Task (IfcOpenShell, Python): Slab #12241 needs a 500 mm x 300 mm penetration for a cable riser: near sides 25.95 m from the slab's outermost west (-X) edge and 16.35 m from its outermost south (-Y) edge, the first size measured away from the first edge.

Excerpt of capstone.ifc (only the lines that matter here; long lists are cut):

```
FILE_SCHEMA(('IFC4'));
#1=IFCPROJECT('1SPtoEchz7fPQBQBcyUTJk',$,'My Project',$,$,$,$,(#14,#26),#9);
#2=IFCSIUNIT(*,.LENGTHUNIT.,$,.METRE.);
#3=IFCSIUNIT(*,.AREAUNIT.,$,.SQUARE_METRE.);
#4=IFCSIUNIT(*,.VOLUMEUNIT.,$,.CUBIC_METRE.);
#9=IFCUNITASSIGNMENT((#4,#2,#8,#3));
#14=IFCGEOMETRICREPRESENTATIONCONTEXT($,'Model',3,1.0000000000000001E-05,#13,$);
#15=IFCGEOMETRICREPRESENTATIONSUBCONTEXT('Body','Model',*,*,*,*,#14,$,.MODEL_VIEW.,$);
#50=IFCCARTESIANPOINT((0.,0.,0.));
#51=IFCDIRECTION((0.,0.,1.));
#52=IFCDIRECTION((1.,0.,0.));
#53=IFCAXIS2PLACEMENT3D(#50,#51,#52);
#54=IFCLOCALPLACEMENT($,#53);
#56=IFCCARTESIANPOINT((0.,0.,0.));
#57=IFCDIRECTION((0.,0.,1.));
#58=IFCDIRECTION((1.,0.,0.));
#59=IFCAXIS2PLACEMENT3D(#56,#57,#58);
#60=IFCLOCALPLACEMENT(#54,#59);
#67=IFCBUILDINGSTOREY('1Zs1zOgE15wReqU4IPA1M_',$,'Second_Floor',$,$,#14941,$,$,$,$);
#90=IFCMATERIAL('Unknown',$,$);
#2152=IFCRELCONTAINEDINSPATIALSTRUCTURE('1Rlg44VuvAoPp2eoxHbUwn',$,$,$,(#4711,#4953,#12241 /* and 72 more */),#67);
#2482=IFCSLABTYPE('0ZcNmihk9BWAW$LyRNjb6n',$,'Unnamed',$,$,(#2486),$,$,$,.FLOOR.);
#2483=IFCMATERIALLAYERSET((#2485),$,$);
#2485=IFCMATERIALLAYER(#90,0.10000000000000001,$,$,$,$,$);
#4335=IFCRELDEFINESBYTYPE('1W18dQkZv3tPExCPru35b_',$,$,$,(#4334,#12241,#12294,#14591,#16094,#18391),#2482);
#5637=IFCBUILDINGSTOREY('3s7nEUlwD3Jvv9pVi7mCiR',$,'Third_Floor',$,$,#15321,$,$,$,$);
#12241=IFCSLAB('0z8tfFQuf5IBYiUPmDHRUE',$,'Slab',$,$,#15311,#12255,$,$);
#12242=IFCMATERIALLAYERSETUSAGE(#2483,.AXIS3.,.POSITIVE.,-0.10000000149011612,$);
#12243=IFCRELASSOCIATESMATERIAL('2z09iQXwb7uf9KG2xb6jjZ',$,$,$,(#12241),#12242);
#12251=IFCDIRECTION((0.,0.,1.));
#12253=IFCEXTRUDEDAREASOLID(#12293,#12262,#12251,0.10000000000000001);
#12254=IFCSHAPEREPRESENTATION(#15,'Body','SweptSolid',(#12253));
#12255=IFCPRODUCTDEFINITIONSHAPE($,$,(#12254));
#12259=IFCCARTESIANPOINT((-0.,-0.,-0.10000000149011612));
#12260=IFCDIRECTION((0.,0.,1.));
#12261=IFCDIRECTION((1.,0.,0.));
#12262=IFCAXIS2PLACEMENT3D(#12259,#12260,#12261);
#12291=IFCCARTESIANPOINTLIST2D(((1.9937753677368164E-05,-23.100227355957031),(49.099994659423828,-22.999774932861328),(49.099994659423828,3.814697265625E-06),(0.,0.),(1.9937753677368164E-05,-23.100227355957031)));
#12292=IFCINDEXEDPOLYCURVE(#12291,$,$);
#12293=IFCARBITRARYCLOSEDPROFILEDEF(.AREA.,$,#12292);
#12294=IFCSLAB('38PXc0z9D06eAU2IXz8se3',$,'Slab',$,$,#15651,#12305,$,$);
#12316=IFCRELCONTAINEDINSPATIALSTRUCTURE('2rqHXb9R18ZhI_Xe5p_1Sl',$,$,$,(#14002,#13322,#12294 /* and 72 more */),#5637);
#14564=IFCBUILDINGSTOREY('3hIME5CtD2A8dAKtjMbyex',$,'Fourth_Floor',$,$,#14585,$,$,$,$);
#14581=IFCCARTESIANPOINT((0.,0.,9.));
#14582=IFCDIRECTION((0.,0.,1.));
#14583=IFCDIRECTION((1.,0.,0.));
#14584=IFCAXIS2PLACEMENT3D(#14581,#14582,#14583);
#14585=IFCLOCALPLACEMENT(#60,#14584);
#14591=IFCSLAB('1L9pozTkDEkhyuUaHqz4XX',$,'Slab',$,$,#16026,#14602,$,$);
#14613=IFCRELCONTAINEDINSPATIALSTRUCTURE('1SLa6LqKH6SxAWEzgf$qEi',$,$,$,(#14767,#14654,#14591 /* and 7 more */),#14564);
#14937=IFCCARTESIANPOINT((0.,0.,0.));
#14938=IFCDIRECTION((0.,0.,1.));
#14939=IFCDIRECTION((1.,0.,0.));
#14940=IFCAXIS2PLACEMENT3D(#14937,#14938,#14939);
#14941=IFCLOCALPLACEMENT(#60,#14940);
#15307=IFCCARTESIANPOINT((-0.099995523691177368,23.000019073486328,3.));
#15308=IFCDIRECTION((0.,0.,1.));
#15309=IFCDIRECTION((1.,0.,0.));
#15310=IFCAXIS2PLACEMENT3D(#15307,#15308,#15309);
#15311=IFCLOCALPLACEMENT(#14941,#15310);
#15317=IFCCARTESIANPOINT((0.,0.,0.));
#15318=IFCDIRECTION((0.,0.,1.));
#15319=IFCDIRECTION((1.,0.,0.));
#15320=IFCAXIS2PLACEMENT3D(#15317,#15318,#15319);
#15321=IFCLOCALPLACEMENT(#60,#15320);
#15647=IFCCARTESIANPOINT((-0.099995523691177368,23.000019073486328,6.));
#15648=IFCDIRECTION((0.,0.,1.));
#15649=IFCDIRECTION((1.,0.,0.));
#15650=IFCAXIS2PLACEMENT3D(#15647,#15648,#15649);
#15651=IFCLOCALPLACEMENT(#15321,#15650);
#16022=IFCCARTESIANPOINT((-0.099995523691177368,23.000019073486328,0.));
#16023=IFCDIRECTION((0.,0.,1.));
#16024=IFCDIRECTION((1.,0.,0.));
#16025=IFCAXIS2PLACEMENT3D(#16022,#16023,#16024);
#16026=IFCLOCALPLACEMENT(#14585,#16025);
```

```python
import numpy as np
import ifcopenshell
import ifcopenshell.api.feature
import ifcopenshell.api.geometry
import ifcopenshell.api.root
import ifcopenshell.geom
import ifcopenshell.util.placement
import ifcopenshell.util.representation
import ifcopenshell.util.shape
import ifcopenshell.util.unit

model = ifcopenshell.open("capstone.ifc")
unit_scale = ifcopenshell.util.unit.calculate_unit_scale(model)
settings = ifcopenshell.geom.settings()


def volume(element):
    """Net volume in cubic metres, openings subtracted."""
    shape = ifcopenshell.geom.create_shape(settings, element)
    return ifcopenshell.util.shape.get_volume(shape.geometry)


slab = model.by_id(12241)
before = volume(slab)

# Extent in the slab's own axes, in metres. The edges named are its -X and -Y sides.
slab_shape = ifcopenshell.geom.create_shape(settings, slab)
vertices = ifcopenshell.util.shape.get_vertices(slab_shape.geometry)
x_min, y_min, bottom = vertices.min(axis=0)
top = vertices[:, 2].max()

opening = ifcopenshell.api.root.create_entity(model, ifc_class="IfcOpeningElement", name="Cable riser opening", predefined_type="OPENING")
context = ifcopenshell.util.representation.get_context(model, "Model", "Body", "MODEL_VIEW")
width, depth = 0.5, 0.3
outline = [(0.0, 0.0), (width, 0.0), (width, depth), (0.0, depth), (0.0, 0.0)]
# Overshoot both faces by 50 mm so the cut is clean.
shape = ifcopenshell.api.geometry.add_slab_representation(
    model, context=context, depth=top - bottom + 0.1, polyline=outline
)
ifcopenshell.api.geometry.assign_representation(model, product=opening, representation=shape)

matrix = ifcopenshell.util.placement.get_local_placement(slab.ObjectPlacement)
matrix[:, 3] = matrix @ np.append(np.array([x_min + 25.95, y_min + 16.35, bottom - 0.05]) / unit_scale, 1.0)
ifcopenshell.api.geometry.edit_object_placement(model, product=opening, matrix=matrix, is_si=False)
ifcopenshell.api.feature.add_feature(model, feature=opening, element=slab)

after = volume(slab)

print(f"slab volume {before:.3f} -> {after:.3f} m3")

model.write("capstone_edited.ifc")
```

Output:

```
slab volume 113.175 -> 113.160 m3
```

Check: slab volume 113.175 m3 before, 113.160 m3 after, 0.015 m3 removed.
